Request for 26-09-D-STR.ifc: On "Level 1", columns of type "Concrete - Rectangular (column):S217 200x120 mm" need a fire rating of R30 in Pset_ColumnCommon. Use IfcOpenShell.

First a look at what the model holds.

```python
import ifcopenshell
import ifcopenshell.util.element

model = ifcopenshell.open("26-09-D-STR.ifc")
print(model.schema)
storey = next(s for s in model.by_type("IfcBuildingStorey") if s.Name == "Level 1")
columns = [e for e in ifcopenshell.util.element.get_decomposition(storey) if e.is_a("IfcColumn")]
seen = {}
for e in columns:
    element_type = ifcopenshell.util.element.get_type(e)
    key = (element_type.Name if element_type != e and element_type else None, ifcopenshell.util.element.get_pset(e, "Pset_ColumnCommon", "FireRating"))
    seen[key] = seen.get(key, 0) + 1
for (name, value), count in sorted(seen.items(), key=str):
    print(count, "x", name, "|", value)
```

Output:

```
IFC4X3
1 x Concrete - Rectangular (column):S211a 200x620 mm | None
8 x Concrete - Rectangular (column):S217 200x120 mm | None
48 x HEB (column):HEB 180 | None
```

```python
import ifcopenshell
import ifcopenshell.api.pset
import ifcopenshell.util.element

model = ifcopenshell.open("26-09-D-STR.ifc")

storey = next(s for s in model.by_type("IfcBuildingStorey") if s.Name == "Level 1")
columns = [e for e in ifcopenshell.util.element.get_decomposition(storey) if e.is_a("IfcColumn")]

count = 0
for e in columns:
    element_type = ifcopenshell.util.element.get_type(e)
    if element_type in (None, e) or element_type.Name != "Concrete - Rectangular (column):S217 200x120 mm":
        continue
    # add_pset returns the element's existing set when there is one.
    pset = ifcopenshell.api.pset.add_pset(model, product=e, name="Pset_ColumnCommon")
    ifcopenshell.api.pset.edit_pset(model, pset=pset, properties={"FireRating": "R30"})
    count += 1

print(count, "columns updated")

model.write("26-09-D-STR-out.ifc")
```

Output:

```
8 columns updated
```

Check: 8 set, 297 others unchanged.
